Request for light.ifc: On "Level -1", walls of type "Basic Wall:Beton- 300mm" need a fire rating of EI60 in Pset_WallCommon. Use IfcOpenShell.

First a look at what the model holds.

```python
import ifcopenshell
import ifcopenshell.util.element

model = ifcopenshell.open("light.ifc")
print(model.schema)
storey = next(s for s in model.by_type("IfcBuildingStorey") if s.Name == "Level -1")
walls = [e for e in ifcopenshell.util.element.get_decomposition(storey) if e.is_a("IfcWall")]
seen = {}
for e in walls:
    element_type = ifcopenshell.util.element.get_type(e)
    key = (element_type.Name if element_type != e and element_type else None, ifcopenshell.util.element.get_pset(e, "Pset_WallCommon", "FireRating"))
    seen[key] = seen.get(key, 0) + 1
for (name, value), count in sorted(seen.items(), key=str):
    print(count, "x", name, "|", value)
```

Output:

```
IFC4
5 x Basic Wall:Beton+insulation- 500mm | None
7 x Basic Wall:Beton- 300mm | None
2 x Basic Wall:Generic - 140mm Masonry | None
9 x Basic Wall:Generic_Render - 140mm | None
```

```python
import ifcopenshell
import ifcopenshell.api.pset
import ifcopenshell.util.element

model = ifcopenshell.open("light.ifc")

storey = next(s for s in model.by_type("IfcBuildingStorey") if s.Name == "Level -1")
walls = [e for e in ifcopenshell.util.element.get_decomposition(storey) if e.is_a("IfcWall")]

count = 0
for e in walls:
    element_type = ifcopenshell.util.element.get_type(e)
    if element_type in (None, e) or element_type.Name != "Basic Wall:Beton- 300mm":
        continue
    # add_pset returns the element's existing set when there is one.
    pset = ifcopenshell.api.pset.add_pset(model, product=e, name="Pset_WallCommon")
    ifcopenshell.api.pset.edit_pset(model, pset=pset, properties={"FireRating": "EI60"})
    count += 1

print(count, "walls updated")

model.write("light_edited.ifc")
```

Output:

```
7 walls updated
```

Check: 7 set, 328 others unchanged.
